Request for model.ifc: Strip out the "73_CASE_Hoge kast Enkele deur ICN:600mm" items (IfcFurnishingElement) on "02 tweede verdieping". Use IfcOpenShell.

First a look at what the model holds.

```python
import ifcopenshell
import ifcopenshell.util.element

model = ifcopenshell.open("model.ifc")
print(model.schema)
storey = next(s for s in model.by_type("IfcBuildingStorey") if s.Name == "02 tweede verdieping")
furniture = [e for e in ifcopenshell.util.element.get_decomposition(storey) if e.is_a("IfcFurnishingElement")]
seen = {}
for e in furniture:
    element_type = ifcopenshell.util.element.get_type(e)
    name = element_type.Name if element_type not in (None, e) else None
    seen[name] = seen.get(name, 0) + 1
for name, count in sorted(seen.items(), key=str):
    print(count, "x", name)
```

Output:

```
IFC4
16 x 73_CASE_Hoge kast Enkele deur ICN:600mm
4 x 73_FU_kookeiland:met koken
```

```python
import ifcopenshell
import ifcopenshell.api.root
import ifcopenshell.util.element

model = ifcopenshell.open("model.ifc")

storey = next(s for s in model.by_type("IfcBuildingStorey") if s.Name == "02 tweede verdieping")
furniture = [e for e in ifcopenshell.util.element.get_decomposition(storey) if e.is_a("IfcFurnishingElement")]
targets = [e for e in furniture if (t := ifcopenshell.util.element.get_type(e)) not in (None, e) and t.Name == "73_CASE_Hoge kast Enkele deur ICN:600mm"]

for e in targets:
    ifcopenshell.api.root.remove_product(model, product=e)
print(len(targets), "removed")

model.write("model_v2.ifc")
```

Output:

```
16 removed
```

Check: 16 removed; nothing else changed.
